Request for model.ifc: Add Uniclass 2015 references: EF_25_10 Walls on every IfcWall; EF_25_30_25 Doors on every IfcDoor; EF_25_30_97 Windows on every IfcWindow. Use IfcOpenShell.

First a look at what the model holds.

```python
import ifcopenshell

model = ifcopenshell.open("model.ifc")
print(model.schema)
print("classifications:", [c.Name for c in model.by_type("IfcClassification")])
for ifc_class in ("IfcDoor", "IfcRoof", "IfcStair", "IfcWall", "IfcWindow"):
    print(ifc_class, len(model.by_type(ifc_class)))
```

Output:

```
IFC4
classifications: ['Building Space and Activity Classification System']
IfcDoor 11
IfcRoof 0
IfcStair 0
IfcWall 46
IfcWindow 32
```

```python
import ifcopenshell
import ifcopenshell.api.classification

model = ifcopenshell.open("model.ifc")

system = ifcopenshell.api.classification.add_classification(model, classification="Uniclass 2015")

codes = {
    "IfcWall": ("EF_25_10", "Walls"),
    "IfcDoor": ("EF_25_30_25", "Doors"),
    "IfcWindow": ("EF_25_30_97", "Windows"),
}
for ifc_class, (code, name) in codes.items():
    products = model.by_type(ifc_class)
    ifcopenshell.api.classification.add_reference(
        model, products=products, classification=system, identification=code, name=name
    )
    print(code, len(products))

model.write("model_updated.ifc")
```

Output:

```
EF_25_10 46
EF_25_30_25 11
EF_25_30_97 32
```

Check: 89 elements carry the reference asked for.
